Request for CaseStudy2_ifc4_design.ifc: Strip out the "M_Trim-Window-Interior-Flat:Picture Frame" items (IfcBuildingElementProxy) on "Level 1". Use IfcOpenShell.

First a look at what the model holds.

```python
import ifcopenshell
import ifcopenshell.util.element

model = ifcopenshell.open("CaseStudy2_ifc4_design.ifc")
print(model.schema)
storey = next(s for s in model.by_type("IfcBuildingStorey") if s.Name == "Level 1")
proxies = [e for e in ifcopenshell.util.element.get_decomposition(storey) if e.is_a("IfcBuildingElementProxy")]
seen = {}
for e in proxies:
    element_type = ifcopenshell.util.element.get_type(e)
    name = element_type.Name if element_type not in (None, e) else None
    seen[name] = seen.get(name, 0) + 1
for name, count in sorted(seen.items(), key=str):
    print(count, "x", name)
```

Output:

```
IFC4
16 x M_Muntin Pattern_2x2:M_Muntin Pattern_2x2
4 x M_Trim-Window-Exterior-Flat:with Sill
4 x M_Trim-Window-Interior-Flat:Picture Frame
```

```python
import ifcopenshell
import ifcopenshell.api.root
import ifcopenshell.util.element

model = ifcopenshell.open("CaseStudy2_ifc4_design.ifc")

storey = next(s for s in model.by_type("IfcBuildingStorey") if s.Name == "Level 1")
proxies = [e for e in ifcopenshell.util.element.get_decomposition(storey) if e.is_a("IfcBuildingElementProxy")]
targets = [e for e in proxies if (t := ifcopenshell.util.element.get_type(e)) not in (None, e) and t.Name == "M_Trim-Window-Interior-Flat:Picture Frame"]

for e in targets:
    ifcopenshell.api.root.remove_product(model, product=e)
print(len(targets), "removed")

model.write("CaseStudy2_ifc4_design_edited.ifc")
```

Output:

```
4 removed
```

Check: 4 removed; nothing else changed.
